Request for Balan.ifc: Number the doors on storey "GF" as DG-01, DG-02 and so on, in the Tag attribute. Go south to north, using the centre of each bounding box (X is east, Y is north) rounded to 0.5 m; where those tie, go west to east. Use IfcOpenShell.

First a look at what the model holds.

```python
import ifcopenshell
import ifcopenshell.util.element
import ifcopenshell.util.placement

model = ifcopenshell.open("Balan.ifc")
print(model.schema)
storey = next(s for s in model.by_type("IfcBuildingStorey") if s.Name == "GF")
doors = [e for e in ifcopenshell.util.element.get_decomposition(storey) if e.is_a("IfcDoor")]
for e in sorted(doors, key=lambda e: e.id()):
    origin = ifcopenshell.util.placement.get_local_placement(e.ObjectPlacement)[:3, 3]
    print(e.id(), e.Tag, e.Name, origin.round(2) + 0.0, sep=" | ")
```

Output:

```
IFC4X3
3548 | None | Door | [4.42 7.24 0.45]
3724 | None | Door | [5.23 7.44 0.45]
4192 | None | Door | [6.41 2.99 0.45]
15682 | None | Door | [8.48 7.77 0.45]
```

```python
import ifcopenshell
import ifcopenshell.geom
import ifcopenshell.util.element
import ifcopenshell.util.shape

model = ifcopenshell.open("Balan.ifc")
settings = ifcopenshell.geom.settings()
settings.set("use-world-coords", True)


def centre(element):
    shape = ifcopenshell.geom.create_shape(settings, element)
    return ifcopenshell.util.shape.get_bbox_centroid(shape.geometry)


storey = next(s for s in model.by_type("IfcBuildingStorey") if s.Name == "GF")
doors = [e for e in ifcopenshell.util.element.get_decomposition(storey) if e.is_a("IfcDoor")]

# Insertion points can sit at a corner or the storey origin, so sort by the geometry (in metres).
centres = {e: centre(e) for e in doors}
doors.sort(key=lambda e: (round(centres[e][1] / 0.5), centres[e][0]))

for i, e in enumerate(doors, start=1):
    number = f"DG-{i:02d}"
    e.Tag = number
    print(e.id(), number)

model.write("Balan_updated.ifc")
```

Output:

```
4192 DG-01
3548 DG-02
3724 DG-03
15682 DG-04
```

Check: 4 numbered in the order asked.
